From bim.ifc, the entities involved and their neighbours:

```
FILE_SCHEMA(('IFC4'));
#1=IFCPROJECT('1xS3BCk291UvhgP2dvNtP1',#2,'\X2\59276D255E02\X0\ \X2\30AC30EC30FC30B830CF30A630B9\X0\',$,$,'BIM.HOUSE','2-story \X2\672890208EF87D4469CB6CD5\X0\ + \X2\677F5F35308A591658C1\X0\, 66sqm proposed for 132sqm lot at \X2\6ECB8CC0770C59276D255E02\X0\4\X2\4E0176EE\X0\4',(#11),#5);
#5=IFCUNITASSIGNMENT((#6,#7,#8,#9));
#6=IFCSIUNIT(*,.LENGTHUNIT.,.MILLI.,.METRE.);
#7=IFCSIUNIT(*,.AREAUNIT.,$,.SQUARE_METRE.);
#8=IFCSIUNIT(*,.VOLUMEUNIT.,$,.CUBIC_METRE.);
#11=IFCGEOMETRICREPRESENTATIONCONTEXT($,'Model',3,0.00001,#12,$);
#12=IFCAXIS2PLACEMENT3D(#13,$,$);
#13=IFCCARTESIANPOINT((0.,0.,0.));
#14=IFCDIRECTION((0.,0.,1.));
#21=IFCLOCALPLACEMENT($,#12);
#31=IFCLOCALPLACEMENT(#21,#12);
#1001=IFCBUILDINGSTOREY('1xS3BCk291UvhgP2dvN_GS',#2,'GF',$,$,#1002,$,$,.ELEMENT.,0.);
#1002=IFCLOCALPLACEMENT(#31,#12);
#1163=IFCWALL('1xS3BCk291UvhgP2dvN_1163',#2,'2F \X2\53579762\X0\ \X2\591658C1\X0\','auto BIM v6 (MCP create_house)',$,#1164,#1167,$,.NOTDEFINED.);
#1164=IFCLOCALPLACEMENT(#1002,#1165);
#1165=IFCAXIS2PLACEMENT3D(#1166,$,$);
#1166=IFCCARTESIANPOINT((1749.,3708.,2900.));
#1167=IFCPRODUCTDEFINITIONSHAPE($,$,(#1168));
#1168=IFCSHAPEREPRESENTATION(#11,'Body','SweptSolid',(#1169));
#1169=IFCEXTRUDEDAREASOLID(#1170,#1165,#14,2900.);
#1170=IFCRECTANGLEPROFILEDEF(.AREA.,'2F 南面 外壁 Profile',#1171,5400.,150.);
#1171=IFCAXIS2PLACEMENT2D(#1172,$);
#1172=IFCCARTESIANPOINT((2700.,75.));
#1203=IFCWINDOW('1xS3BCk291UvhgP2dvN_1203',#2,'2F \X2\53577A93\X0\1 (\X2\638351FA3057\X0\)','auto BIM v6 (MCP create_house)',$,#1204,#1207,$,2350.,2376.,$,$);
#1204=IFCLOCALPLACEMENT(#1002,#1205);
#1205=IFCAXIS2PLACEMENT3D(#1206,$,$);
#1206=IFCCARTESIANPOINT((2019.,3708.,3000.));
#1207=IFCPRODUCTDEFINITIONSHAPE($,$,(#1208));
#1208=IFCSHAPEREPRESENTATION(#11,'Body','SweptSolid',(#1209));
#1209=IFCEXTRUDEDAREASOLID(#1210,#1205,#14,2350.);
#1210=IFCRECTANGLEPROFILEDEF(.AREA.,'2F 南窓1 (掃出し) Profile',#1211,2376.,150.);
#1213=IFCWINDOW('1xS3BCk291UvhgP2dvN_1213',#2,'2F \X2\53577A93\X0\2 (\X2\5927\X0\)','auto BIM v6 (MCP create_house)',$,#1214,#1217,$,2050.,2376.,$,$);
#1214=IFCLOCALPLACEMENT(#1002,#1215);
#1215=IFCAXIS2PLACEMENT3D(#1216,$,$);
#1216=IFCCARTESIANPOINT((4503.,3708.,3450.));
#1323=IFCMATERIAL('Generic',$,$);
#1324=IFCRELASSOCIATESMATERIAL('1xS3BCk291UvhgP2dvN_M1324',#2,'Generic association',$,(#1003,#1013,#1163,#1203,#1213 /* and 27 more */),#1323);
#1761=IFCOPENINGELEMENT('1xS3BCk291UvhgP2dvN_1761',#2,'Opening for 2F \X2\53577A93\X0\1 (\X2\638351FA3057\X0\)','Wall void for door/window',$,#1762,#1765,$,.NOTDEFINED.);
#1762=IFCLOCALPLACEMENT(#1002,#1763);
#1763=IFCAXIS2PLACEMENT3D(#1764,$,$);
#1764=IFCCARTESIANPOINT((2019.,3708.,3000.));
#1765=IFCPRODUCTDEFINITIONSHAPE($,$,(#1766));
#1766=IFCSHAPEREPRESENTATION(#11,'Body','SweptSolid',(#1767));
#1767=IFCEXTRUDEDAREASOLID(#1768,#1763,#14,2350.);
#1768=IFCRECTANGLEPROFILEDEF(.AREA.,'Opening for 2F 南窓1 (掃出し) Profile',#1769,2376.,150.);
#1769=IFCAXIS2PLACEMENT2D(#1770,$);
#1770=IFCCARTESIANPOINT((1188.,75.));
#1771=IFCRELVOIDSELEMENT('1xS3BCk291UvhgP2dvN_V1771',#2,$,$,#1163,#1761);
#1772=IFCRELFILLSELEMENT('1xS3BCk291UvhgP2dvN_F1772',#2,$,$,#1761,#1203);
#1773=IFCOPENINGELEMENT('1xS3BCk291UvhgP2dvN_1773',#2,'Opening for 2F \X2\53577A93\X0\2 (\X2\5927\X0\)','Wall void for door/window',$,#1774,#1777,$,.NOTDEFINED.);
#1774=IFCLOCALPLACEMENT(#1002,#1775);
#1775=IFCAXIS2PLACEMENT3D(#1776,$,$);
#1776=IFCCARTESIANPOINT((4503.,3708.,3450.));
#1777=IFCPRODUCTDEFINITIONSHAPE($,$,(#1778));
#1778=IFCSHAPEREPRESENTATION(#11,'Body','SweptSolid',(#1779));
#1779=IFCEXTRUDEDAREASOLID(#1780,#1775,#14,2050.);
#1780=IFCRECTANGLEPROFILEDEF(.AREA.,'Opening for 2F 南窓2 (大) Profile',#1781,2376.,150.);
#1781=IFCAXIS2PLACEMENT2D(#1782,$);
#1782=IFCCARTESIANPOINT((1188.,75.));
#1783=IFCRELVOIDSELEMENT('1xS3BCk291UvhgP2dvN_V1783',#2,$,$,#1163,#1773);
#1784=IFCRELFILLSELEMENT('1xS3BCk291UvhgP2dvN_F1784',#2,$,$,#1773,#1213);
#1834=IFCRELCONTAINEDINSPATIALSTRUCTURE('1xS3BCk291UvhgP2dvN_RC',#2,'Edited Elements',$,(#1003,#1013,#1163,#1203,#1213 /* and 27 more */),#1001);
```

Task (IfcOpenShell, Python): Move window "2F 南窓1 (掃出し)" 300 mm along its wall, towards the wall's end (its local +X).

```python
import ifcopenshell
import ifcopenshell.api.geometry
import ifcopenshell.util.placement
import ifcopenshell.util.unit

model = ifcopenshell.open("bim.ifc")
unit_scale = ifcopenshell.util.unit.calculate_unit_scale(model)

window = model.by_guid("1xS3BCk291UvhgP2dvN_1203")
opening = window.FillsVoids[0].RelatingOpeningElement
wall = opening.VoidsElements[0].RelatingBuildingElement

wall_matrix = ifcopenshell.util.placement.get_local_placement(wall.ObjectPlacement)
shift = wall_matrix[:3, 0] * 0.3 / unit_scale
before = ifcopenshell.util.placement.get_local_placement(window.ObjectPlacement)[:3, 3].copy()

# The window is not placed relative to its opening, so move both.
for product in (opening, window):
    matrix = ifcopenshell.util.placement.get_local_placement(product.ObjectPlacement)
    matrix[:3, 3] += shift
    ifcopenshell.api.geometry.edit_object_placement(model, product=product, matrix=matrix, is_si=False)

after = ifcopenshell.util.placement.get_local_placement(window.ObjectPlacement)[:3, 3]
print("window moved by", (after - before).round(3) + 0.0)

model.write("bim_updated.ifc")
```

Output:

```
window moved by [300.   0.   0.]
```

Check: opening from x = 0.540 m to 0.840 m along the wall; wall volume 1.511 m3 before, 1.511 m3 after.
